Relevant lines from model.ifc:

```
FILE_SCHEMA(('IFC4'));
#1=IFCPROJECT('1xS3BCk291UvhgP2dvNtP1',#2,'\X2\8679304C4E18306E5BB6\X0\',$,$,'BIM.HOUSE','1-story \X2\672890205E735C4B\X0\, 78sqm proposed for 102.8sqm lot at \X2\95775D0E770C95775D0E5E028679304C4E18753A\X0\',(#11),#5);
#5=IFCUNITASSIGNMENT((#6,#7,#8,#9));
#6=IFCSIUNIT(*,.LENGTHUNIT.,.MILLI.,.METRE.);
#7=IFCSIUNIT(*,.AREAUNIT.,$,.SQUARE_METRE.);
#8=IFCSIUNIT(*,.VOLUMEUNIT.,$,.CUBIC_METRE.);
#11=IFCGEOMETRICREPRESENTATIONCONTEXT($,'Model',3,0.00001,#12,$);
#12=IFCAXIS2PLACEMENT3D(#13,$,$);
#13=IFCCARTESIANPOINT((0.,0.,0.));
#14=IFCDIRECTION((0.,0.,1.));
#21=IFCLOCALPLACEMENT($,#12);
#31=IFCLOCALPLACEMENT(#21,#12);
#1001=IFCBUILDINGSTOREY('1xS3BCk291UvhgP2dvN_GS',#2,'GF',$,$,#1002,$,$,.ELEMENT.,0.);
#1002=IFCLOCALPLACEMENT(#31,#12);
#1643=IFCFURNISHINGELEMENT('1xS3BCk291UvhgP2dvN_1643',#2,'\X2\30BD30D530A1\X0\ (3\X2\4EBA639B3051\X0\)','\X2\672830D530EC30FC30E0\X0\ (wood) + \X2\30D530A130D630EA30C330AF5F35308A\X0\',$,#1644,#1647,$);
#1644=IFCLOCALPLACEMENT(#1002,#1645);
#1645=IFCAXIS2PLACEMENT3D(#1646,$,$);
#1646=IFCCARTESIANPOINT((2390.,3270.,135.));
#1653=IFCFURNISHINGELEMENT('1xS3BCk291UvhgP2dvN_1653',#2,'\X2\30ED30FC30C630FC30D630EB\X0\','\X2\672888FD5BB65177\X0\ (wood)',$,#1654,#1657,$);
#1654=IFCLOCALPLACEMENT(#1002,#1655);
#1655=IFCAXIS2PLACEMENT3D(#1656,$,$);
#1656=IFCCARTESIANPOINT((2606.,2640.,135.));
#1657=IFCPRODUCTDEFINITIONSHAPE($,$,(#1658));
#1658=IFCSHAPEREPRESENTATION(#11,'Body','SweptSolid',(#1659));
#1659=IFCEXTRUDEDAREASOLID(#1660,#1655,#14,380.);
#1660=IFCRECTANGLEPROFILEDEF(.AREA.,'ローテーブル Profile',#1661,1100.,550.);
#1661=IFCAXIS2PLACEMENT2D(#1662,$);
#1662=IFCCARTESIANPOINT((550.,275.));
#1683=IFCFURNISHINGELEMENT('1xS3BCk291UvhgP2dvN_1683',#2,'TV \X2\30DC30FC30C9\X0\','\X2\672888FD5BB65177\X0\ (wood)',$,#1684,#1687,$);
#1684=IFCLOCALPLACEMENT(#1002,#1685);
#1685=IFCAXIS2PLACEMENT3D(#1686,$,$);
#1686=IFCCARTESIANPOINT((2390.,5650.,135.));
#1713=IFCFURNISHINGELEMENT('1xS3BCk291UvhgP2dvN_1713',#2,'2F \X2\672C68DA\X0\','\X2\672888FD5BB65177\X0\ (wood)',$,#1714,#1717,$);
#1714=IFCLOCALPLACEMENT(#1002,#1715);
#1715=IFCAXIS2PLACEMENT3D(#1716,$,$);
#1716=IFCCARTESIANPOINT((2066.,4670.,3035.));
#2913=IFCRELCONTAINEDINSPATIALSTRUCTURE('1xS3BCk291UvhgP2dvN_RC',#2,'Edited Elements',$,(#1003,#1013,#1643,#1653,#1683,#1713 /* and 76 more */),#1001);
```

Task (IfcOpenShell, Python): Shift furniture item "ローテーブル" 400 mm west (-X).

```python
import ifcopenshell
import ifcopenshell.api.geometry
import ifcopenshell.util.placement
import ifcopenshell.util.unit

model = ifcopenshell.open("model.ifc")
unit_scale = ifcopenshell.util.unit.calculate_unit_scale(model)

item = model.by_guid("1xS3BCk291UvhgP2dvN_1653")
matrix = ifcopenshell.util.placement.get_local_placement(item.ObjectPlacement)
matrix[0, 3] -= 0.4 / unit_scale
ifcopenshell.api.geometry.edit_object_placement(model, product=item, matrix=matrix, is_si=False)

print(ifcopenshell.util.placement.get_local_placement(item.ObjectPlacement).round(3) + 0.0)

model.write("model_edited.ifc")
```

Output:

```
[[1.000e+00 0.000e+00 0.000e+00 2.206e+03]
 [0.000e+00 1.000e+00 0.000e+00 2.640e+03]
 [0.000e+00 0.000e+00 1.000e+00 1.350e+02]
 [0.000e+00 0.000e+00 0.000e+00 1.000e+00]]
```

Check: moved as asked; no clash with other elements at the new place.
